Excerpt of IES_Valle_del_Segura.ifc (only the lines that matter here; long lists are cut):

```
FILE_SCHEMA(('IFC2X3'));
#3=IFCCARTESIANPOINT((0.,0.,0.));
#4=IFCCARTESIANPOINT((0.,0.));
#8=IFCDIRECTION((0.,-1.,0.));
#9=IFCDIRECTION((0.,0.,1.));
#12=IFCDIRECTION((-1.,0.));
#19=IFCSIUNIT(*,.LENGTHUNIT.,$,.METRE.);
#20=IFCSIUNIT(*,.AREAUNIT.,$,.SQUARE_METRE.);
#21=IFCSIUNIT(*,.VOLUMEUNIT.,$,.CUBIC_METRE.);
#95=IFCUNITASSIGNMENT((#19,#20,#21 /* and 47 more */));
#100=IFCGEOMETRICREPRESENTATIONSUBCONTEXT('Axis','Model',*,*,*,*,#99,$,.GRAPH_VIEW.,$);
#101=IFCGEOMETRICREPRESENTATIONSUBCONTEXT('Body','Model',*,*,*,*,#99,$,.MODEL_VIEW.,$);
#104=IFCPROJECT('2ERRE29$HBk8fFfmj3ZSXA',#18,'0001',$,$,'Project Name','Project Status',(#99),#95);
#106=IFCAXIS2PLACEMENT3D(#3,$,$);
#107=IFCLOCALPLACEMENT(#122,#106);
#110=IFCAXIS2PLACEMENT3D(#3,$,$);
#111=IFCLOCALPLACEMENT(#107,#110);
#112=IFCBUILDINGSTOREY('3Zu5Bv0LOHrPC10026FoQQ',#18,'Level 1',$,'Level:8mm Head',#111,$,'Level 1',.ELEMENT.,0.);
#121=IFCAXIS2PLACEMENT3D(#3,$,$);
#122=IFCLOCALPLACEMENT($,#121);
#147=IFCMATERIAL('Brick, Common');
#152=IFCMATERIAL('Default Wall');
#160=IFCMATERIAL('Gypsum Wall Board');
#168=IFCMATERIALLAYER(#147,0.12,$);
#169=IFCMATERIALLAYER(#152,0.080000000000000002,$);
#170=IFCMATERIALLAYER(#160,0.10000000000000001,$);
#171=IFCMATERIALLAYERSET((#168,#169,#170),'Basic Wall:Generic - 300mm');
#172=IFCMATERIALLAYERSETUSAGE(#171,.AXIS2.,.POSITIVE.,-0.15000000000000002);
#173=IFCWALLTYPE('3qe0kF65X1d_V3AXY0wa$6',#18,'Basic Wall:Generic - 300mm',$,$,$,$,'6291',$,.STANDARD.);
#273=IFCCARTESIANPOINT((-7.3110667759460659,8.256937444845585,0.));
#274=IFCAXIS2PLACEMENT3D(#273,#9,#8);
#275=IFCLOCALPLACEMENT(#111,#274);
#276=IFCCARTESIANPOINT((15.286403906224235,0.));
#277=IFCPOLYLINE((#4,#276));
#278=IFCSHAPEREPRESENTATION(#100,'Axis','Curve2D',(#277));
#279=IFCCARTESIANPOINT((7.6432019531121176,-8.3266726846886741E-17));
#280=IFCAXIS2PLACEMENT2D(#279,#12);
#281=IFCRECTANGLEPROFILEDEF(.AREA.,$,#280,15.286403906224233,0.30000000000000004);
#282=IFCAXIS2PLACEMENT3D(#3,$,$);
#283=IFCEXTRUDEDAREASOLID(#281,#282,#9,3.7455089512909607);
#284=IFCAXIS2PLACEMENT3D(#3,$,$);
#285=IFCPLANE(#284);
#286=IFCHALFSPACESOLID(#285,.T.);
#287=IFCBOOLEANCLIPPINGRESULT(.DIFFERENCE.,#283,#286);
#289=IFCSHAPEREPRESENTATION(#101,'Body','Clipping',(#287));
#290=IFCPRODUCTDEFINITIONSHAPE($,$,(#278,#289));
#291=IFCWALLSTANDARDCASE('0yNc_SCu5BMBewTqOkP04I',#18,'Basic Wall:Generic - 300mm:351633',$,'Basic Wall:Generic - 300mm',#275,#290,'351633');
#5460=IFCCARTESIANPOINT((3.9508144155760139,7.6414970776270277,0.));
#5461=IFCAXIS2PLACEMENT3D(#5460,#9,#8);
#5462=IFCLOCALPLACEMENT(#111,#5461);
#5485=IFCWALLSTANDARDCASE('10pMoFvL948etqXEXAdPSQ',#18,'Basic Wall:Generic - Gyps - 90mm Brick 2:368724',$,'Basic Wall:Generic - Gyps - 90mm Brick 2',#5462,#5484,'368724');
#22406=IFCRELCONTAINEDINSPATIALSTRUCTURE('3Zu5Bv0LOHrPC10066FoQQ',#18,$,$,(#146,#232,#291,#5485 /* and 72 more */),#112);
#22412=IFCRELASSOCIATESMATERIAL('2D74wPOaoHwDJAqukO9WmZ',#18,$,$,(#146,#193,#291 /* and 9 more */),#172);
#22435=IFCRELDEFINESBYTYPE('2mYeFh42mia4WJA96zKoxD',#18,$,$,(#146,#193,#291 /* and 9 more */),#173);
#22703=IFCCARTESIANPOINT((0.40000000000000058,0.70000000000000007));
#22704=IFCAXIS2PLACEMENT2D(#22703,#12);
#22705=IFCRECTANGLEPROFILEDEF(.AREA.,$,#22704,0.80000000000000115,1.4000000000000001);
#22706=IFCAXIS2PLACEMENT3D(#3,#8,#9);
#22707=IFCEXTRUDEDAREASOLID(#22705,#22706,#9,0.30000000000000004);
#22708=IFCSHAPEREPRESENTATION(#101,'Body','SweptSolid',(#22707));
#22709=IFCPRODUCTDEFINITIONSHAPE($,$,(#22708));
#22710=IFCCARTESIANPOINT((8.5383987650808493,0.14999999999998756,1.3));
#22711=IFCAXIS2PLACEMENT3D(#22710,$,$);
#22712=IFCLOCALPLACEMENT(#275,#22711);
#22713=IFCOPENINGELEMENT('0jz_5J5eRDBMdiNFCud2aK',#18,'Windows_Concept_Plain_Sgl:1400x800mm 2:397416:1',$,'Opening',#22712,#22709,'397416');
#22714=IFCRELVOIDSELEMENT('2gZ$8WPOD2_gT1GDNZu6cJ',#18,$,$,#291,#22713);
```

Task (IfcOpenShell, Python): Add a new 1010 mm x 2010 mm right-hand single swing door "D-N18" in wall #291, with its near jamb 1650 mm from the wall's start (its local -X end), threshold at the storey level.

```python
import numpy as np
import ifcopenshell
import ifcopenshell.api.feature
import ifcopenshell.api.geometry
import ifcopenshell.api.root
import ifcopenshell.api.spatial
import ifcopenshell.api.type
import ifcopenshell.geom
import ifcopenshell.util.element
import ifcopenshell.util.placement
import ifcopenshell.util.representation
import ifcopenshell.util.shape
import ifcopenshell.util.unit

model = ifcopenshell.open("IES_Valle_del_Segura.ifc")
unit_scale = ifcopenshell.util.unit.calculate_unit_scale(model)
settings = ifcopenshell.geom.settings()


def volume(element):
    """Net volume in cubic metres, openings subtracted."""
    shape = ifcopenshell.geom.create_shape(settings, element)
    return ifcopenshell.util.shape.get_volume(shape.geometry)


wall = model.by_guid("0yNc_SCu5BMBewTqOkP04I")
storey = ifcopenshell.util.element.get_container(wall, ifc_class="IfcBuildingStorey")
context = ifcopenshell.util.representation.get_context(model, "Model", "Body", "MODEL_VIEW")
before = volume(wall)

width, height, from_end, sill = 1.01, 2.01, 1.65, 0.0  # metres

# The wall runs along its own X axis, and the end named is its -X end.
wall_shape = ifcopenshell.geom.create_shape(settings, wall)
x, y, z = ifcopenshell.util.shape.get_vertices(wall_shape.geometry).T
start = x.min() + from_end
face, thickness = float(y.min()), float(y.max() - y.min())
wall_matrix = ifcopenshell.util.placement.get_local_placement(wall.ObjectPlacement)
level = ifcopenshell.util.placement.get_local_placement(storey.ObjectPlacement)[2, 3]


def in_wall(x, y):
    """Placement at x, y metres in the wall's axes, at sill height."""
    matrix = wall_matrix.copy()
    matrix[:, 3] = wall_matrix @ np.array([x / unit_scale, y / unit_scale, 0.0, 1.0])
    matrix[2, 3] = level + sill / unit_scale
    return matrix


# Opening: a box that overshoots both wall faces by 50 mm.
opening = ifcopenshell.api.root.create_entity(model, ifc_class="IfcOpeningElement")
box = ifcopenshell.api.geometry.add_wall_representation(
    model, context=context, length=width, height=height, thickness=thickness + 0.1
)
ifcopenshell.api.geometry.assign_representation(model, product=opening, representation=box)
ifcopenshell.api.geometry.edit_object_placement(model, product=opening, matrix=in_wall(start, face - 0.05), is_si=False)
ifcopenshell.api.feature.add_feature(model, feature=opening, element=wall)

door = ifcopenshell.api.root.create_entity(model, ifc_class="IfcDoor", name="D-N18")
door.OverallWidth, door.OverallHeight = width / unit_scale, height / unit_scale
body = ifcopenshell.api.geometry.add_door_representation(
    model,
    context=context,
    overall_width=door.OverallWidth,
    overall_height=door.OverallHeight,
    operation_type="SINGLE_SWING_RIGHT",
    lining_properties={"LiningDepth": thickness / unit_scale, "ThresholdDepth": thickness / unit_scale},
)
ifcopenshell.api.geometry.assign_representation(model, product=door, representation=body)
ifcopenshell.api.spatial.assign_container(model, products=[door], relating_structure=storey)
fills = ifcopenshell.api.feature.add_filling(model, opening=opening, element=door)
fills.OwnerHistory = door.OwnerHistory  # required in IFC2X3

# IFC2X3 keeps the operation on the door style.
style = ifcopenshell.api.root.create_entity(model, ifc_class="IfcDoorStyle", name="D-N18")
style.OperationType, style.ConstructionType = "SINGLE_SWING_RIGHT", "NOTDEFINED"
style.ParameterTakesPrecedence = style.Sizeable = False
ifcopenshell.api.type.assign_type(model, related_objects=[door], relating_type=style)

# The lining spans the wall, so the door starts at the wall face.
ifcopenshell.api.geometry.edit_object_placement(model, product=door, matrix=in_wall(start, face), is_si=False)

after = volume(wall)

print(f"wall volume {before:.3f} -> {after:.3f} m3")

model.write("IES_Valle_del_Segura_edited.ifc")
```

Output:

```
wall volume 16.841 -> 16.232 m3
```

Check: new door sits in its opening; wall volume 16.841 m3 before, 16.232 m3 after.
